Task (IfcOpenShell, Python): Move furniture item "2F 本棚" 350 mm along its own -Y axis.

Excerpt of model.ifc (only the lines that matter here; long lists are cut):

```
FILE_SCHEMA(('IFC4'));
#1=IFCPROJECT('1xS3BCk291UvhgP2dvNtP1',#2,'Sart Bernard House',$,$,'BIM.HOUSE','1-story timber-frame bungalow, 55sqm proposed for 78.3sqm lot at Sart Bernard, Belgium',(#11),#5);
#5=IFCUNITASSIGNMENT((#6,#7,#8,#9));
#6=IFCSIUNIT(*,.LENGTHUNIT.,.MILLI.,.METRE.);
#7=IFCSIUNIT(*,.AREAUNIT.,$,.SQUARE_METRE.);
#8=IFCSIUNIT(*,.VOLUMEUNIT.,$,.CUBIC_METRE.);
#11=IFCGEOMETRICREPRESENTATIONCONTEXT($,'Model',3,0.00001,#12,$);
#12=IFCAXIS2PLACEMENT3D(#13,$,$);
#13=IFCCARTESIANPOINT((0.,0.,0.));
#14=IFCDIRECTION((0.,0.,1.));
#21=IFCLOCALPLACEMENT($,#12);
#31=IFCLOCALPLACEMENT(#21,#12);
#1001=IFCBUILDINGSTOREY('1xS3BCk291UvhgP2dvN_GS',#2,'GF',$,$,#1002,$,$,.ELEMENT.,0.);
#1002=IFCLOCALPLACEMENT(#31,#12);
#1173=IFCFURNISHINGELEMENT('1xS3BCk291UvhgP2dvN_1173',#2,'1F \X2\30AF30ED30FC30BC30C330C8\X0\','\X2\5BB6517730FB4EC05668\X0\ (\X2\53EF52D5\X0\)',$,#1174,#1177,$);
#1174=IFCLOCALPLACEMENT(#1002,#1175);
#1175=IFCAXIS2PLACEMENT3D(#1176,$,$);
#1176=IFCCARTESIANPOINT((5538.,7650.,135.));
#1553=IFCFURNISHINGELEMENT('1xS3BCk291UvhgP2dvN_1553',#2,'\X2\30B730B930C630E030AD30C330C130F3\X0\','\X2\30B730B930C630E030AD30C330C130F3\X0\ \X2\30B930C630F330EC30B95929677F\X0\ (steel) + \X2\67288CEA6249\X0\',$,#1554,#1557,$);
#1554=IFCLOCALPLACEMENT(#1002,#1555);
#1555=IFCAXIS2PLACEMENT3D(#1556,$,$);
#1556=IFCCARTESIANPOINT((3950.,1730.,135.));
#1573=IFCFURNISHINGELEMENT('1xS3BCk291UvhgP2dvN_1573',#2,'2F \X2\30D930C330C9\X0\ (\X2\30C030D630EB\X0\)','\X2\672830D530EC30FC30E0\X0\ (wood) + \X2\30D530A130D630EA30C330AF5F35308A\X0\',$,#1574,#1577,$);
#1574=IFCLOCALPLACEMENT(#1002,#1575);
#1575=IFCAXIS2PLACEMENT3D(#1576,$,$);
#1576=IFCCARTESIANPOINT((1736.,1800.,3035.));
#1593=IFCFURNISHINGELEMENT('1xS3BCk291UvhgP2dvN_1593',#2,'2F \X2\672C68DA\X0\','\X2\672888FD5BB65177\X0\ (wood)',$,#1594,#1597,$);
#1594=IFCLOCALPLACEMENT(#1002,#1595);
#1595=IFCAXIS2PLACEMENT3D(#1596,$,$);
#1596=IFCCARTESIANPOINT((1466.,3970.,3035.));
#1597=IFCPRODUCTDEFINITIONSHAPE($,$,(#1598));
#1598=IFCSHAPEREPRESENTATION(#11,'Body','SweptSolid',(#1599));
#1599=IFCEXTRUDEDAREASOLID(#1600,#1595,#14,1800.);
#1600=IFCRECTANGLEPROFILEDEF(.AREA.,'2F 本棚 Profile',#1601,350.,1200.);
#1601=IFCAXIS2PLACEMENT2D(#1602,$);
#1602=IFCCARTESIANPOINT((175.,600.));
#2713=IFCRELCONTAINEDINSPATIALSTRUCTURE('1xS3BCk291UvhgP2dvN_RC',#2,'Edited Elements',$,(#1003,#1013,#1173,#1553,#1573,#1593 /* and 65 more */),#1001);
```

```python
import ifcopenshell
import ifcopenshell.api.geometry
import ifcopenshell.util.placement
import ifcopenshell.util.unit

model = ifcopenshell.open("model.ifc")
unit_scale = ifcopenshell.util.unit.calculate_unit_scale(model)

item = model.by_guid("1xS3BCk291UvhgP2dvN_1593")
matrix = ifcopenshell.util.placement.get_local_placement(item.ObjectPlacement)
matrix[:3, 3] -= matrix[:3, 1] * 0.35 / unit_scale
ifcopenshell.api.geometry.edit_object_placement(model, product=item, matrix=matrix, is_si=False)

print(ifcopenshell.util.placement.get_local_placement(item.ObjectPlacement).round(3) + 0.0)

model.write("model_rev.ifc")
```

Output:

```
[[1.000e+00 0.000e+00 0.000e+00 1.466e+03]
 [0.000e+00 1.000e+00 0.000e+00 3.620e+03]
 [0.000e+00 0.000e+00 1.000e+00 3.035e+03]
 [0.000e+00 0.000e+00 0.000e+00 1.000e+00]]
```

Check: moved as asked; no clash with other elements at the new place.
